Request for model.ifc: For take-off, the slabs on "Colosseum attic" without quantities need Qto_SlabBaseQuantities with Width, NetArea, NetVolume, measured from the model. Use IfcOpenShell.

First a look at what the model holds.

```python
import ifcopenshell
import ifcopenshell.util.element
import ifcopenshell.util.unit

model = ifcopenshell.open("model.ifc")
print(model.schema)
for unit_type in ("LENGTHUNIT", "AREAUNIT", "VOLUMEUNIT"):
    print(unit_type, ifcopenshell.util.unit.calculate_unit_scale(model, unit_type))
storey = next(s for s in model.by_type("IfcBuildingStorey") if s.Name == "Colosseum attic")
slabs = [e for e in ifcopenshell.util.element.get_decomposition(storey) if e.is_a("IfcSlab")]
for e in sorted(slabs, key=lambda e: e.id()):
    print(e.id(), e.is_a(), e.Name, list(ifcopenshell.util.element.get_psets(e, qtos_only=True)), sep=" | ")
```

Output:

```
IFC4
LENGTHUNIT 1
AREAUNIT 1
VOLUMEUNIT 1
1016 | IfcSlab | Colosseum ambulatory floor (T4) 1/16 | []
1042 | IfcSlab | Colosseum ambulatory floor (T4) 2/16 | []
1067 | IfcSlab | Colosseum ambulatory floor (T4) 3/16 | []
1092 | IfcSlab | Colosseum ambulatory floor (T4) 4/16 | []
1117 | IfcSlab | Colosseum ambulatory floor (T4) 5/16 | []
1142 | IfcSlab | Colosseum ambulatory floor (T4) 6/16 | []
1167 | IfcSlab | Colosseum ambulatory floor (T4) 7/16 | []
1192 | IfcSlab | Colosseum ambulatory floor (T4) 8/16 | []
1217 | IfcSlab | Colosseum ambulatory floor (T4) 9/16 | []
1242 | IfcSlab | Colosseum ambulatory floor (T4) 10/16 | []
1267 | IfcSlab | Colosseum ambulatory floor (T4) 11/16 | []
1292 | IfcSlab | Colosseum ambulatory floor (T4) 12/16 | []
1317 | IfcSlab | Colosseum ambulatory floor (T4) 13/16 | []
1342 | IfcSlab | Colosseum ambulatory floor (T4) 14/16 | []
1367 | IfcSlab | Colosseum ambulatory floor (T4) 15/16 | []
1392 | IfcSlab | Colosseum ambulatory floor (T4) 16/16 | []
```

```python
import ifcopenshell
import ifcopenshell.api.pset
import ifcopenshell.geom
import ifcopenshell.util.element
import ifcopenshell.util.shape
import ifcopenshell.util.unit

model = ifcopenshell.open("model.ifc")
unit_scale = ifcopenshell.util.unit.calculate_unit_scale(model)
area_scale = ifcopenshell.util.unit.calculate_unit_scale(model, "AREAUNIT")
volume_scale = ifcopenshell.util.unit.calculate_unit_scale(model, "VOLUMEUNIT")
settings = ifcopenshell.geom.settings()

storey = next(s for s in model.by_type("IfcBuildingStorey") if s.Name == "Colosseum attic")
slabs = [e for e in ifcopenshell.util.element.get_decomposition(storey) if e.is_a("IfcSlab")]

for e in sorted(slabs, key=lambda e: e.id()):
    if ifcopenshell.util.element.get_psets(e, qtos_only=True, should_inherit=False):
        continue
    # Geometry comes back in metres, in the element's own axes.
    shape = ifcopenshell.geom.create_shape(settings, e)
    values = {
        "Width": ifcopenshell.util.shape.get_z(shape.geometry) / unit_scale,
        "NetArea": ifcopenshell.util.shape.get_footprint_area(shape.geometry) / area_scale,
        "NetVolume": ifcopenshell.util.shape.get_volume(shape.geometry) / volume_scale,
    }
    qto = ifcopenshell.api.pset.add_qto(model, product=e, name="Qto_SlabBaseQuantities")
    ifcopenshell.api.pset.edit_qto(model, qto=qto, properties=values)
    print(e.id(), {k: round(v, 3) for k, v in values.items()})

model.write("model_rev.ifc")
```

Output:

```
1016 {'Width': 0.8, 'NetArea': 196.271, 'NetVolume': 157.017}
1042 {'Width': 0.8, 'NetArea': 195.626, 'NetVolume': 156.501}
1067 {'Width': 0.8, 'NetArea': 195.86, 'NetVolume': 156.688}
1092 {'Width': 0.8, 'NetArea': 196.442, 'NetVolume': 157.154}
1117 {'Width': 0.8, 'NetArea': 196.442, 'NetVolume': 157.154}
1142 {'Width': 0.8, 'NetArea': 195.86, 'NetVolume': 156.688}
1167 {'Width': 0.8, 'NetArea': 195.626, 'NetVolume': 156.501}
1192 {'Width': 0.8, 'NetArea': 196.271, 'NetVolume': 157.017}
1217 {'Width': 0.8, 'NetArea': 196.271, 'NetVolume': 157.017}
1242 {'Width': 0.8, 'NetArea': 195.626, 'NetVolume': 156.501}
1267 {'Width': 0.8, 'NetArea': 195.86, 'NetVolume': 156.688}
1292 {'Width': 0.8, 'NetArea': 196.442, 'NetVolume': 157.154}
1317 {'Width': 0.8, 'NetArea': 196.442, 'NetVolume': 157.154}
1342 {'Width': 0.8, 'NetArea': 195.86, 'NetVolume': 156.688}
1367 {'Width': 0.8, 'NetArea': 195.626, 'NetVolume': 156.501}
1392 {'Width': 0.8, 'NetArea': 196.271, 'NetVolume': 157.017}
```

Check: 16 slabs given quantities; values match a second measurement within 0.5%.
